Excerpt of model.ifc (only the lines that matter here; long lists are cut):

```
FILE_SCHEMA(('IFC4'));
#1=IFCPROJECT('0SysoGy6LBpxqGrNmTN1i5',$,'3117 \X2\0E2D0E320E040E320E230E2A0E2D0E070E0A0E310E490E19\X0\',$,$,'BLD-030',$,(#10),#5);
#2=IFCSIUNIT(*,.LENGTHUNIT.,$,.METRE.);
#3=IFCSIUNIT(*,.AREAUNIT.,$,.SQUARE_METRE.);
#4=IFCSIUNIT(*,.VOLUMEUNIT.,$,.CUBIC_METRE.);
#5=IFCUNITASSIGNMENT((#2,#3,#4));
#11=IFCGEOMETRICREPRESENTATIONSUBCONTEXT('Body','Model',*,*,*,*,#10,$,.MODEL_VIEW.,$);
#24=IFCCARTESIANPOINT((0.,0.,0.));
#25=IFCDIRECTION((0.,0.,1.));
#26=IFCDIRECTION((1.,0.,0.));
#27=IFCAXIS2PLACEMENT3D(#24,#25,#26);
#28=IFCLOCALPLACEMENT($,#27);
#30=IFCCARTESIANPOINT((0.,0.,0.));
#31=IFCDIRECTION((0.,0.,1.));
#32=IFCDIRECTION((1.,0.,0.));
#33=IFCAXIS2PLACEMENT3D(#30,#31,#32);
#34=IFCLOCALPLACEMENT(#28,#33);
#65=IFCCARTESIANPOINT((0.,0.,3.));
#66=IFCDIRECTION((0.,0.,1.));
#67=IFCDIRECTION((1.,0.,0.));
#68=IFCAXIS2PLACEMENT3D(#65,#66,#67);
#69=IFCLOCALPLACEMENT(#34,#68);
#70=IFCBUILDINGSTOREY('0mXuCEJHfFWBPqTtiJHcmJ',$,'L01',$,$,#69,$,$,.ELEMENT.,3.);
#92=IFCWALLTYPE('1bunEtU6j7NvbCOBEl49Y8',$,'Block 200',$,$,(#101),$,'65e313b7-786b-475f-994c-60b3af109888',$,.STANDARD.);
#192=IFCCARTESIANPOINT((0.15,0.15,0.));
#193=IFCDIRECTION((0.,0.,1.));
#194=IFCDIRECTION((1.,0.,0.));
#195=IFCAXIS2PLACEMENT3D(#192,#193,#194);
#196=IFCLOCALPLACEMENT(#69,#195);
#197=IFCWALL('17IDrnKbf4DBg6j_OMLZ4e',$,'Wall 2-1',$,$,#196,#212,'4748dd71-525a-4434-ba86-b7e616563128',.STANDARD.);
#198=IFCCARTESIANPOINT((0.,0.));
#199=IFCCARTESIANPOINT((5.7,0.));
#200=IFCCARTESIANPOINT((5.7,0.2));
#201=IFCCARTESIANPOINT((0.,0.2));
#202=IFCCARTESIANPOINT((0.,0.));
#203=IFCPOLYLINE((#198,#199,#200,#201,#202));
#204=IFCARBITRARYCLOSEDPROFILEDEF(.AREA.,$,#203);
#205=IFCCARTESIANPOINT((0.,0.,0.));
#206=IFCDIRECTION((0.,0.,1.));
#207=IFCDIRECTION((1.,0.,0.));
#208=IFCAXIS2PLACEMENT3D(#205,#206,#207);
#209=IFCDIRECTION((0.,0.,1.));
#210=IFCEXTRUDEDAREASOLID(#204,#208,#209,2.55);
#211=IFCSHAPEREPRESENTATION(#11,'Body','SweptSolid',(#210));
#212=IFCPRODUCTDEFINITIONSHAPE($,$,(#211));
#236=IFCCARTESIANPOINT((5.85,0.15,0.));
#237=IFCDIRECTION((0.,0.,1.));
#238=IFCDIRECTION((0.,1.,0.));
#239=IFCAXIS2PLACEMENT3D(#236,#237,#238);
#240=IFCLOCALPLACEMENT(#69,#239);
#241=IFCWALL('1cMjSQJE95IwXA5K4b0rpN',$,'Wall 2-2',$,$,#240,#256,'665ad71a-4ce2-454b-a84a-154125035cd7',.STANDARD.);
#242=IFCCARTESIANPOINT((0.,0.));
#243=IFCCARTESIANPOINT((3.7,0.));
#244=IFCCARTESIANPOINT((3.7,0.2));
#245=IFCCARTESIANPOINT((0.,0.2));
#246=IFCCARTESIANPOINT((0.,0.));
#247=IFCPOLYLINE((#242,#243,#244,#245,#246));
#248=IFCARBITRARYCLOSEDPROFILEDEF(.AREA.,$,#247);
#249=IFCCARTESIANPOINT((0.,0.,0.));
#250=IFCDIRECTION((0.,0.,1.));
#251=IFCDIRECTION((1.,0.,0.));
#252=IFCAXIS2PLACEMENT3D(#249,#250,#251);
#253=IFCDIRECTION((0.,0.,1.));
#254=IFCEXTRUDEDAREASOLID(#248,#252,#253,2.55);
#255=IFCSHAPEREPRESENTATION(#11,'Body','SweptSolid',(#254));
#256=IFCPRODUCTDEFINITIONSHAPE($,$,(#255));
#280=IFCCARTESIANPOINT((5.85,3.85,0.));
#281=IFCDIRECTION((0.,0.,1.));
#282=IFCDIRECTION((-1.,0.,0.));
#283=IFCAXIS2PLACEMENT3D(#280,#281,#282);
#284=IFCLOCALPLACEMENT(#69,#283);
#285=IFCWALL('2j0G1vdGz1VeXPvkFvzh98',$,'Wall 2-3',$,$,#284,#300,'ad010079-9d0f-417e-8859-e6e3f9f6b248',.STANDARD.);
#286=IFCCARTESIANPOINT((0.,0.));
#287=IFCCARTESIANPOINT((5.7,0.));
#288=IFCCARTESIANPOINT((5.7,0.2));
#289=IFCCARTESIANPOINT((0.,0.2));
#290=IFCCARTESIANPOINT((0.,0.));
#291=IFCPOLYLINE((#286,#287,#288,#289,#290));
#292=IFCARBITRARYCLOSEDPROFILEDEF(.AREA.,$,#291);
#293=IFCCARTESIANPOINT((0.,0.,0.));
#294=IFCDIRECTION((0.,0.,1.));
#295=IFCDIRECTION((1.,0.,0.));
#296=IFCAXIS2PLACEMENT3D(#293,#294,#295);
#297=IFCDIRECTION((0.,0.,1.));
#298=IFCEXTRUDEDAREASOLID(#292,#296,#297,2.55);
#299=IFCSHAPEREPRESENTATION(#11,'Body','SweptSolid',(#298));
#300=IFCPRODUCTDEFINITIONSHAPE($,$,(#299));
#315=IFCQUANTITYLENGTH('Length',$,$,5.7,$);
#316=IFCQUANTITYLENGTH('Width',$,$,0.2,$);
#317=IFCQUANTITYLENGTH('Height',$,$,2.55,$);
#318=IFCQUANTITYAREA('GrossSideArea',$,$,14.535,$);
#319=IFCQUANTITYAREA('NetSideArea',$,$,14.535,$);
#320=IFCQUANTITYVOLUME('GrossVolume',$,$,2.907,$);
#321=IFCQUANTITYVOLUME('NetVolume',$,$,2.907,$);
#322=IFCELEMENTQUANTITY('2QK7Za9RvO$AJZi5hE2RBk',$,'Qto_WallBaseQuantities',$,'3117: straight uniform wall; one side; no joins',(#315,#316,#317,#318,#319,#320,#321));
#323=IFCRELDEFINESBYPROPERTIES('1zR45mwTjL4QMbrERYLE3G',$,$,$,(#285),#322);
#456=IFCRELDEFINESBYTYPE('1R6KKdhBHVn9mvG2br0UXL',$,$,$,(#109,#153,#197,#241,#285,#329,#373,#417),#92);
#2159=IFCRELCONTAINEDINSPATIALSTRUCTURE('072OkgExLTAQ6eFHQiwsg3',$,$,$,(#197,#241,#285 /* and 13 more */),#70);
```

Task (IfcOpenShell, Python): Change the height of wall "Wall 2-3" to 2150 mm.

```python
import ifcopenshell
import ifcopenshell.api.pset
import ifcopenshell.geom
import ifcopenshell.util.element
import ifcopenshell.util.representation
import ifcopenshell.util.shape
import ifcopenshell.util.unit

model = ifcopenshell.open("model.ifc")
unit_scale = ifcopenshell.util.unit.calculate_unit_scale(model)
area_scale = ifcopenshell.util.unit.calculate_unit_scale(model, "AREAUNIT")
volume_scale = ifcopenshell.util.unit.calculate_unit_scale(model, "VOLUMEUNIT")
settings = ifcopenshell.geom.settings()


def volume(element):
    """Net volume in cubic metres, openings subtracted."""
    shape = ifcopenshell.geom.create_shape(settings, element)
    return ifcopenshell.util.shape.get_volume(shape.geometry)


wall = model.by_guid("2j0G1vdGz1VeXPvkFvzh98")
before = volume(wall)

body = ifcopenshell.util.representation.get_representation(wall, "Model", "Body")
solid = body.Items[0]
old_height = solid.Depth
solid.Depth = 2.15 / unit_scale
after = volume(wall)
thickness = 0.2  # wall thickness in metres

# Update the stored height, areas and volumes.
qto = model.by_id(ifcopenshell.util.element.get_pset(wall, "Qto_WallBaseQuantities", should_inherit=False)["id"])
ifcopenshell.api.pset.edit_qto(model, qto=qto, properties={
    "Height": solid.Depth,
    "GrossSideArea": ifcopenshell.util.element.get_pset(wall, "Qto_WallBaseQuantities", "GrossSideArea") * solid.Depth / old_height,
    "NetSideArea": after / thickness / area_scale,
    "GrossVolume": ifcopenshell.util.element.get_pset(wall, "Qto_WallBaseQuantities", "GrossVolume") * solid.Depth / old_height,
    "NetVolume": after / volume_scale,
})

print(f"height {old_height:g} -> {solid.Depth:g}, volume {before:.3f} -> {after:.3f} m3")

model.write("model-out.ifc")
```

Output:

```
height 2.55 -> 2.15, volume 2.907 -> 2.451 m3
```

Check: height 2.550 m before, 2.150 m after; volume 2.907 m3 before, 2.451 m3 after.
